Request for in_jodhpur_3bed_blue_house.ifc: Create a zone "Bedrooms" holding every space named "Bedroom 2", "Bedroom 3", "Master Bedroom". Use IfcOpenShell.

First a look at what the model holds.

```python
import ifcopenshell

model = ifcopenshell.open("in_jodhpur_3bed_blue_house.ifc")
print(model.schema)
seen = {}
for space in model.by_type("IfcSpace"):
    seen[space.LongName] = seen.get(space.LongName, 0) + 1
for name, count in sorted(seen.items(), key=str):
    print(count, "x", name)
print("zones:", [z.Name for z in model.by_type("IfcZone")][:20])
```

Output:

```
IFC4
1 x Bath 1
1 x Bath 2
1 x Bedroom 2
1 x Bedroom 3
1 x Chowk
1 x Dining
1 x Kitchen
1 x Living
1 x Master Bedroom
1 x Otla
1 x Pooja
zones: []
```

```python
import ifcopenshell
import ifcopenshell.api.group
import ifcopenshell.api.root

model = ifcopenshell.open("in_jodhpur_3bed_blue_house.ifc")

names = {"Bedroom 2", "Bedroom 3", "Master Bedroom"}
spaces = [s for s in model.by_type("IfcSpace") if s.LongName in names]

zone = ifcopenshell.api.root.create_entity(model, ifc_class="IfcZone", name="Bedrooms")
ifcopenshell.api.group.assign_group(model, products=spaces, group=zone)
print(len(spaces), "spaces in", zone.Name)

model.write("in_jodhpur_3bed_blue_house_rev.ifc")
```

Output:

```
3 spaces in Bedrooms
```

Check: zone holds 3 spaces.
